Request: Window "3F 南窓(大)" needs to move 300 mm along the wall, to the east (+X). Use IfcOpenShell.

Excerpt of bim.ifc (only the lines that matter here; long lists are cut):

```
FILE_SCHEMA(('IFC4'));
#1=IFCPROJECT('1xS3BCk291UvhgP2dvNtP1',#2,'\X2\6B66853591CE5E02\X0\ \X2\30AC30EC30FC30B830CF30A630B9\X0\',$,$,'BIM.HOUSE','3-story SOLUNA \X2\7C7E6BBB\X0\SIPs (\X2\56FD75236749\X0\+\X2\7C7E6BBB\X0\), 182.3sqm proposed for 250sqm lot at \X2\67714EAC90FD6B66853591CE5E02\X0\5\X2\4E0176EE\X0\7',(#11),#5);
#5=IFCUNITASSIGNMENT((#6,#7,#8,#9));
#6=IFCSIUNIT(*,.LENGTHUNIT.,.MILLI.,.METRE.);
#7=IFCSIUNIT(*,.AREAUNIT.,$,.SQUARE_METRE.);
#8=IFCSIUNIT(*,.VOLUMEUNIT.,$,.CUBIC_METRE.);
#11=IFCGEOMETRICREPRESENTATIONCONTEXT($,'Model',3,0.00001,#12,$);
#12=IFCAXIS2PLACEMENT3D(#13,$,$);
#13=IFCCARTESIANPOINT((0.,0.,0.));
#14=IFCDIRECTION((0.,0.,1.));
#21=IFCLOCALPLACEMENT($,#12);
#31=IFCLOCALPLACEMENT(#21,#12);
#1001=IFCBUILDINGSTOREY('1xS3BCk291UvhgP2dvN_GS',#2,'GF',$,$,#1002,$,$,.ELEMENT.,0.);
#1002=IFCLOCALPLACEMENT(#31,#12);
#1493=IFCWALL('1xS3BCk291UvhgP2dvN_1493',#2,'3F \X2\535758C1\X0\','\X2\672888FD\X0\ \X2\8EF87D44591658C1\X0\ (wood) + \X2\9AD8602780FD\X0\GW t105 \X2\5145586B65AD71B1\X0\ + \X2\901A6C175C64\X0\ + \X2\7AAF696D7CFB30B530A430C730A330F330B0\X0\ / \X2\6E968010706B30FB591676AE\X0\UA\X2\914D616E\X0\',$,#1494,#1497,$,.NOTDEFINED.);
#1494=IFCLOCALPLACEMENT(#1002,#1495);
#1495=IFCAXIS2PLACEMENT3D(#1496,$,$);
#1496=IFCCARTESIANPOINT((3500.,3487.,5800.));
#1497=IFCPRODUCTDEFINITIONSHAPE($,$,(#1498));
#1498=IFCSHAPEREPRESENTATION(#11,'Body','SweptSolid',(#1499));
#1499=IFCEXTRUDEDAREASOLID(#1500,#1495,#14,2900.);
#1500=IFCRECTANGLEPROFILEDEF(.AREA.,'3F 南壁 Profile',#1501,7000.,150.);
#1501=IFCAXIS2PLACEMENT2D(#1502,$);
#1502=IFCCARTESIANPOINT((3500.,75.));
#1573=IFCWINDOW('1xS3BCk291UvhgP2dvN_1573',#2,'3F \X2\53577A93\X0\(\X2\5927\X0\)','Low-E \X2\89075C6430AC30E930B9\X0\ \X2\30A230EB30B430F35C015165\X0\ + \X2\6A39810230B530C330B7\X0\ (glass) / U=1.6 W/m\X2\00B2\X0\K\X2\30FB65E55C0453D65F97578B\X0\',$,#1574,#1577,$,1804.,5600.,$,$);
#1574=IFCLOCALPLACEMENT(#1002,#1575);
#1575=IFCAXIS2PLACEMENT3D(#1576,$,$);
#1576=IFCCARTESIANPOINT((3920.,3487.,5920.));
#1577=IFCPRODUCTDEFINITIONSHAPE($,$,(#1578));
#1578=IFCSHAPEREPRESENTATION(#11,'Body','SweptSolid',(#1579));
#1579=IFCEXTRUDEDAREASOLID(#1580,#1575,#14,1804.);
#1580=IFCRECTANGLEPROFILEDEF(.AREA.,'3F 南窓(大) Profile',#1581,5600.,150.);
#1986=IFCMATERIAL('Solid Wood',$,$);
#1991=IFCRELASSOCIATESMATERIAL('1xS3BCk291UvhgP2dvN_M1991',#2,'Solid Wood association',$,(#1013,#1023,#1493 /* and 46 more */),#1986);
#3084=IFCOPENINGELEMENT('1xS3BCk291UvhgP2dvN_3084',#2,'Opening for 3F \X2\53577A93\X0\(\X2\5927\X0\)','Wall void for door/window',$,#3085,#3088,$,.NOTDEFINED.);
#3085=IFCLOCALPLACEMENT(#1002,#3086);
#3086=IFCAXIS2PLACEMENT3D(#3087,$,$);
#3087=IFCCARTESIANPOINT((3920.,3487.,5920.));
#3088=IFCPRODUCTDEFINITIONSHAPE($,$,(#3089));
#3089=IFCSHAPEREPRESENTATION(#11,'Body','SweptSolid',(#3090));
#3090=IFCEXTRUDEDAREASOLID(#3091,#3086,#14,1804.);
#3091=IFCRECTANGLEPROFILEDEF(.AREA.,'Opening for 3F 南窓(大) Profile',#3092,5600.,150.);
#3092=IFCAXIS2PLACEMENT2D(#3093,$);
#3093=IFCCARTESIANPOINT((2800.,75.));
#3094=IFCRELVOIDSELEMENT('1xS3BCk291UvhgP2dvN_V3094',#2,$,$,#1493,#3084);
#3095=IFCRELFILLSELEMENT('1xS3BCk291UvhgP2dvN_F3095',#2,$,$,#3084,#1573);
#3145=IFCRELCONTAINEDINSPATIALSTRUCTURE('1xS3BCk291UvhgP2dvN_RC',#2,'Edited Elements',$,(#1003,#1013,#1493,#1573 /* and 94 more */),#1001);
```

```python
import ifcopenshell
import ifcopenshell.api.geometry
import ifcopenshell.util.placement

model = ifcopenshell.open("bim.ifc")

window = model.by_guid("1xS3BCk291UvhgP2dvN_1573")
opening = window.FillsVoids[0].RelatingOpeningElement
wall = opening.VoidsElements[0].RelatingBuildingElement

wall_matrix = ifcopenshell.util.placement.get_local_placement(wall.ObjectPlacement)
shift = wall_matrix[:3, 0] * 300.0
before = ifcopenshell.util.placement.get_local_placement(window.ObjectPlacement)[:3, 3].copy()

# The window is not placed relative to its opening, so move both.
for product in (opening, window):
    matrix = ifcopenshell.util.placement.get_local_placement(product.ObjectPlacement)
    matrix[:3, 3] += shift
    ifcopenshell.api.geometry.edit_object_placement(model, product=product, matrix=matrix, is_si=False)

after = ifcopenshell.util.placement.get_local_placement(window.ObjectPlacement)[:3, 3]
print("window moved by", (after - before).round(3) + 0.0)

model.write("bim-out.ifc")
```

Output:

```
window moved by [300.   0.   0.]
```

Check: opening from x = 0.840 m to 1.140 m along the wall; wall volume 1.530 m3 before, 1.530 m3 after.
